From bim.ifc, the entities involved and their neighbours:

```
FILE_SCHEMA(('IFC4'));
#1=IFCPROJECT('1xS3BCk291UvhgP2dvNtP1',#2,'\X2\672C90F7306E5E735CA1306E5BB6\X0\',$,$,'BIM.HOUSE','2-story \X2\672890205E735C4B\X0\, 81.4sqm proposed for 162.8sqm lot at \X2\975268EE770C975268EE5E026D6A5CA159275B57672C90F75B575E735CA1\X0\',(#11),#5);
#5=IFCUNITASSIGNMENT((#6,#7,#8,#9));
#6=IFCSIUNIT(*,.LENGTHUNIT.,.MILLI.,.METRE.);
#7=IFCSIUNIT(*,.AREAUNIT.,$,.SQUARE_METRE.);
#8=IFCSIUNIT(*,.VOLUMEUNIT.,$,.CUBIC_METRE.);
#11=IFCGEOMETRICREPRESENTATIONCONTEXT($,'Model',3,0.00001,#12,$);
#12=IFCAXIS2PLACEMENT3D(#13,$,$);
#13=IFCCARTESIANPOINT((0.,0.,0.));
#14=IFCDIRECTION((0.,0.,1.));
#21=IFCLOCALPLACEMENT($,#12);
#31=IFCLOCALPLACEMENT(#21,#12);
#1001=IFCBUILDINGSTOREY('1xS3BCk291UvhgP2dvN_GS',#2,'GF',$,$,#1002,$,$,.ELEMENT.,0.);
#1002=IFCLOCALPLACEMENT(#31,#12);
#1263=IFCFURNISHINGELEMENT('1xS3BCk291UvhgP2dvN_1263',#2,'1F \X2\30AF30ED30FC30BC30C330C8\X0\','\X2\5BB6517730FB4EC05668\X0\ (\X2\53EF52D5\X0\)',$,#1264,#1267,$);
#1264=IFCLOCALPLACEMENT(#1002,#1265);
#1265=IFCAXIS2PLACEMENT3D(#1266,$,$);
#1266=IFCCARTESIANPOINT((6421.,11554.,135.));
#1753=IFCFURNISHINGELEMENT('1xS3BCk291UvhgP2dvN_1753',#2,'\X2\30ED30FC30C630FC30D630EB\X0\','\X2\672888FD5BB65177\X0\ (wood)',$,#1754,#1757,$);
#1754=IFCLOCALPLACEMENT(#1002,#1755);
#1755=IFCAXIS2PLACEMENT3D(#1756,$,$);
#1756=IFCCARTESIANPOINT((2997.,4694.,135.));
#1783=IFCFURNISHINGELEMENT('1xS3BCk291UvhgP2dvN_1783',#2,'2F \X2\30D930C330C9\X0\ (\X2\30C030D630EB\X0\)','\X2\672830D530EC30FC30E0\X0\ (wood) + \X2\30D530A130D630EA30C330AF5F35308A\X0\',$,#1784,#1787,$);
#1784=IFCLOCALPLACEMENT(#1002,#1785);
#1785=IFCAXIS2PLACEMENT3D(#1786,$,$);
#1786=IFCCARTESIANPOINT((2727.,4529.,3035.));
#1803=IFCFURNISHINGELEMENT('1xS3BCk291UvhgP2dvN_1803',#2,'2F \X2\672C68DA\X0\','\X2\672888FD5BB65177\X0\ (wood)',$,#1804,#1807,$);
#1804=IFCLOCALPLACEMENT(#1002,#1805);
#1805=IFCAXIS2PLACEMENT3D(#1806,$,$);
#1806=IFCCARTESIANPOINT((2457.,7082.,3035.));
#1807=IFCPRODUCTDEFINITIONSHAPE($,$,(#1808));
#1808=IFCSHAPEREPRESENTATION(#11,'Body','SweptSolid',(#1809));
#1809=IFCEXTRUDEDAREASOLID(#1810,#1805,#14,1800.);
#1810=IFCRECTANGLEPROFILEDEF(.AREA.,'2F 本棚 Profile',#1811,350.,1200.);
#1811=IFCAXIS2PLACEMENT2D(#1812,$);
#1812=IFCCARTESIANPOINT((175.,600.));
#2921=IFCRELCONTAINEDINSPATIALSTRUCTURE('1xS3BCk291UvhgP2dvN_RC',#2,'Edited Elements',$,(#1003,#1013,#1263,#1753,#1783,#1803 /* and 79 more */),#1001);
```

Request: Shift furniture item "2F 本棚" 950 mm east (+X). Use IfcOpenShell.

```python
import ifcopenshell
import ifcopenshell.api.geometry
import ifcopenshell.util.placement

model = ifcopenshell.open("bim.ifc")

item = model.by_guid("1xS3BCk291UvhgP2dvN_1803")
matrix = ifcopenshell.util.placement.get_local_placement(item.ObjectPlacement)
matrix[0, 3] += 950.0
ifcopenshell.api.geometry.edit_object_placement(model, product=item, matrix=matrix, is_si=False)

print(ifcopenshell.util.placement.get_local_placement(item.ObjectPlacement).round(3) + 0.0)

model.write("bim_v2.ifc")
```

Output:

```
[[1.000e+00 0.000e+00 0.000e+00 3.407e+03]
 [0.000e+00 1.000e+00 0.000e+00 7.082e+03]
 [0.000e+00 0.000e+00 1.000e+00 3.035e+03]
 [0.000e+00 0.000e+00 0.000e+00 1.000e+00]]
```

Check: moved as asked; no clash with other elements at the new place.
